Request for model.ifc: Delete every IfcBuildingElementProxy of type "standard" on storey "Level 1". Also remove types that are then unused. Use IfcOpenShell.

First a look at what the model holds.

```python
import ifcopenshell
import ifcopenshell.util.element

model = ifcopenshell.open("model.ifc")
print(model.schema)
storey = next(s for s in model.by_type("IfcBuildingStorey") if s.Name == "Level 1")
proxies = [e for e in ifcopenshell.util.element.get_decomposition(storey) if e.is_a("IfcBuildingElementProxy")]
seen = {}
for e in proxies:
    element_type = ifcopenshell.util.element.get_type(e)
    name = element_type.Name if element_type not in (None, e) else None
    seen[name] = seen.get(name, 0) + 1
for name, count in sorted(seen.items(), key=str):
    print(count, "x", name)
```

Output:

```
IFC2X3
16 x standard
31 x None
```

```python
import ifcopenshell
import ifcopenshell.api.root
import ifcopenshell.util.element

model = ifcopenshell.open("model.ifc")

storey = next(s for s in model.by_type("IfcBuildingStorey") if s.Name == "Level 1")
proxies = [e for e in ifcopenshell.util.element.get_decomposition(storey) if e.is_a("IfcBuildingElementProxy")]
targets = [e for e in proxies if (t := ifcopenshell.util.element.get_type(e)) not in (None, e) and t.Name == "standard"]
types = {ifcopenshell.util.element.get_type(e) for e in targets} - {None, *targets}

for e in targets:
    ifcopenshell.api.root.remove_product(model, product=e)
print(len(targets), "removed")

unused = [t for t in types if not ifcopenshell.util.element.get_types(t)]
for t in unused:
    ifcopenshell.api.root.remove_product(model, product=t)
print(len(unused), "unused types removed")

model.write("model_rev.ifc")
```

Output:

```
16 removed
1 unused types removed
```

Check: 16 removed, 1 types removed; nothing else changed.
